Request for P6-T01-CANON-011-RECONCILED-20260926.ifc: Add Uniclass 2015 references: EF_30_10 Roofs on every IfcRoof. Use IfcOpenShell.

First a look at what the model holds.

```python
import ifcopenshell

model = ifcopenshell.open("P6-T01-CANON-011-RECONCILED-20260926.ifc")
print(model.schema)
print("classifications:", [c.Name for c in model.by_type("IfcClassification")])
for ifc_class in ("IfcDoor", "IfcRoof", "IfcStair", "IfcWall", "IfcWindow"):
    print(ifc_class, len(model.by_type(ifc_class)))
```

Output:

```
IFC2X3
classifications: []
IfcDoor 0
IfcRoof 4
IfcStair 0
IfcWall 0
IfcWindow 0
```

```python
import ifcopenshell
import ifcopenshell.api.classification

model = ifcopenshell.open("P6-T01-CANON-011-RECONCILED-20260926.ifc")

# IFC2X3 requires Source and Edition and has no link from the project to the system.
system = model.create_entity("IfcClassification", Source="NBS", Edition="2015", Name="Uniclass 2015")

codes = {
    "IfcRoof": ("EF_30_10", "Roofs"),
}
for ifc_class, (code, name) in codes.items():
    products = model.by_type(ifc_class)
    ifcopenshell.api.classification.add_reference(
        model, products=products, classification=system, identification=code, name=name
    )
    print(code, len(products))

model.write("P6-T01-CANON-011-RECONCILED-20260926_v2.ifc")
```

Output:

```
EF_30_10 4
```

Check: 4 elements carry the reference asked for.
